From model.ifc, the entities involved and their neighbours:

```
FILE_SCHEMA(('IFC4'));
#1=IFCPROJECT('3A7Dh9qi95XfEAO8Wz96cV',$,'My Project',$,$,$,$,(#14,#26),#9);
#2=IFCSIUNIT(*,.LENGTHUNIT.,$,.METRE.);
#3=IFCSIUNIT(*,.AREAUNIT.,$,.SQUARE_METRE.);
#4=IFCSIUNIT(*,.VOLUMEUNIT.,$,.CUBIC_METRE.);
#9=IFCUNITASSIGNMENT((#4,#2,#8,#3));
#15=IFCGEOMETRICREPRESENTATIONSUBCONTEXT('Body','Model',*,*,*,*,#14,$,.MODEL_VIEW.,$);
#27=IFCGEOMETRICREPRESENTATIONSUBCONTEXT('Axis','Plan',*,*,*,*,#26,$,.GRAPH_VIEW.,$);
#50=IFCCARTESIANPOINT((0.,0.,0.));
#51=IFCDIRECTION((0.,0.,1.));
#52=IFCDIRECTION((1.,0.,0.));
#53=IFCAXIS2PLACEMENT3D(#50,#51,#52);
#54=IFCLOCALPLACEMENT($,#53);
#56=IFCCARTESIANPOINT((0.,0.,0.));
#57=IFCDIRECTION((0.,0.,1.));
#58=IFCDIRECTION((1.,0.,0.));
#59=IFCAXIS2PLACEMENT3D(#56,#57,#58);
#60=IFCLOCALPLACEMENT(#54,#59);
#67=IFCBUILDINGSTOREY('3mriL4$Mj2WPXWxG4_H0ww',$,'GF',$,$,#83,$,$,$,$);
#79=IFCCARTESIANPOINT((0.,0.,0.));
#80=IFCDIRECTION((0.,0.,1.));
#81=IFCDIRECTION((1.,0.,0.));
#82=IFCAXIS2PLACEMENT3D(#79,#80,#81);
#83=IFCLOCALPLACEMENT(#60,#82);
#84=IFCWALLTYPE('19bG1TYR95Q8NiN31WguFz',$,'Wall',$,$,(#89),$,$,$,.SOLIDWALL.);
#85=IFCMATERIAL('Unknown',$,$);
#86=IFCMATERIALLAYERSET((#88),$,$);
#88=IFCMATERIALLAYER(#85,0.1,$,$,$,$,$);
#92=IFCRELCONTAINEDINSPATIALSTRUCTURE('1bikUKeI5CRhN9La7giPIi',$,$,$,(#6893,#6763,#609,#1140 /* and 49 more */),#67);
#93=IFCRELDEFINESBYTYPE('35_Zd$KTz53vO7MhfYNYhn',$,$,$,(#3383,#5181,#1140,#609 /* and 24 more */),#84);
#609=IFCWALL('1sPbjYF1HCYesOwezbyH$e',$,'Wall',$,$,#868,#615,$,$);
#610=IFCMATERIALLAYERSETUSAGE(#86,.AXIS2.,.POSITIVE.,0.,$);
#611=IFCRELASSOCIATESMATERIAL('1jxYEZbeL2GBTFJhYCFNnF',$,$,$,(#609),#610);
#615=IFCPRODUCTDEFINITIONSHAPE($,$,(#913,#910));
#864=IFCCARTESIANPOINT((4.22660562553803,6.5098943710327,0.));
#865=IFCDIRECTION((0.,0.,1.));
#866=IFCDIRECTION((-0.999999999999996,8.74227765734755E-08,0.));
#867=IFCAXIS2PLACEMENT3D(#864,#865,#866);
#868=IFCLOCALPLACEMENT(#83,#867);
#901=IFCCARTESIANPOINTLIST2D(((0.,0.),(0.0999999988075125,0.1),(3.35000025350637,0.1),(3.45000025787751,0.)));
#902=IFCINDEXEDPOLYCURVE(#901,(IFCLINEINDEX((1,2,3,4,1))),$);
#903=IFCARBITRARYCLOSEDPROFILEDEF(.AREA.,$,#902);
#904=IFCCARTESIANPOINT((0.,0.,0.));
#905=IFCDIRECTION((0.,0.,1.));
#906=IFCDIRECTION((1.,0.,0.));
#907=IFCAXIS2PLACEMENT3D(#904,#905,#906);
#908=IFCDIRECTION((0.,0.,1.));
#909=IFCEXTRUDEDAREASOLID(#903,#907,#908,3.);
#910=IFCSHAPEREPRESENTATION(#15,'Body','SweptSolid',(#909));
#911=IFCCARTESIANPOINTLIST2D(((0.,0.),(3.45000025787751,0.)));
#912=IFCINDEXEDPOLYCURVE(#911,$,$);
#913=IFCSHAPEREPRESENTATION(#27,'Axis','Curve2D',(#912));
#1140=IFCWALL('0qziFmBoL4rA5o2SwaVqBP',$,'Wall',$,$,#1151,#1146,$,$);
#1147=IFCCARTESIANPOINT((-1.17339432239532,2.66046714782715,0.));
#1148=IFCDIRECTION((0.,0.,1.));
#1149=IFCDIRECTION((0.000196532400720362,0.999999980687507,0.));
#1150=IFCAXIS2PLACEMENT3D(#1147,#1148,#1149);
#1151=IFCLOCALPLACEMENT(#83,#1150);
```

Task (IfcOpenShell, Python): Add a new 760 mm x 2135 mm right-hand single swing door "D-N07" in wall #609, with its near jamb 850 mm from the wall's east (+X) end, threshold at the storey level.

```python
import numpy as np
import ifcopenshell
import ifcopenshell.api.feature
import ifcopenshell.api.geometry
import ifcopenshell.api.root
import ifcopenshell.api.spatial
import ifcopenshell.geom
import ifcopenshell.util.element
import ifcopenshell.util.placement
import ifcopenshell.util.representation
import ifcopenshell.util.shape
import ifcopenshell.util.unit

model = ifcopenshell.open("model.ifc")
unit_scale = ifcopenshell.util.unit.calculate_unit_scale(model)
settings = ifcopenshell.geom.settings()


def volume(element):
    """Net volume in cubic metres, openings subtracted."""
    shape = ifcopenshell.geom.create_shape(settings, element)
    return ifcopenshell.util.shape.get_volume(shape.geometry)


wall = model.by_guid("1sPbjYF1HCYesOwezbyH$e")
storey = ifcopenshell.util.element.get_container(wall, ifc_class="IfcBuildingStorey")
context = ifcopenshell.util.representation.get_context(model, "Model", "Body", "MODEL_VIEW")
before = volume(wall)

width, height, from_end, sill = 0.76, 2.135, 0.85, 0.0  # metres

# The wall runs along its own X axis, and the end named is its -X end.
wall_shape = ifcopenshell.geom.create_shape(settings, wall)
x, y, z = ifcopenshell.util.shape.get_vertices(wall_shape.geometry).T
start = x.min() + from_end
face, thickness = float(y.min()), float(y.max() - y.min())
wall_matrix = ifcopenshell.util.placement.get_local_placement(wall.ObjectPlacement)
level = ifcopenshell.util.placement.get_local_placement(storey.ObjectPlacement)[2, 3]


def in_wall(x, y):
    """Placement at x, y metres in the wall's axes, at sill height."""
    matrix = wall_matrix.copy()
    matrix[:, 3] = wall_matrix @ np.array([x / unit_scale, y / unit_scale, 0.0, 1.0])
    matrix[2, 3] = level + sill / unit_scale
    return matrix


# Opening: a box that overshoots both wall faces by 50 mm.
opening = ifcopenshell.api.root.create_entity(model, ifc_class="IfcOpeningElement", predefined_type="OPENING")
box = ifcopenshell.api.geometry.add_wall_representation(
    model, context=context, length=width, height=height, thickness=thickness + 0.1
)
ifcopenshell.api.geometry.assign_representation(model, product=opening, representation=box)
ifcopenshell.api.geometry.edit_object_placement(model, product=opening, matrix=in_wall(start, face - 0.05), is_si=False)
ifcopenshell.api.feature.add_feature(model, feature=opening, element=wall)

door = ifcopenshell.api.root.create_entity(model, ifc_class="IfcDoor", name="D-N07", predefined_type="DOOR")
door.OverallWidth, door.OverallHeight = width / unit_scale, height / unit_scale
door.OperationType = "SINGLE_SWING_RIGHT"
body = ifcopenshell.api.geometry.add_door_representation(
    model,
    context=context,
    overall_width=door.OverallWidth,
    overall_height=door.OverallHeight,
    operation_type="SINGLE_SWING_RIGHT",
    lining_properties={"LiningDepth": thickness / unit_scale, "ThresholdDepth": thickness / unit_scale},
)
ifcopenshell.api.geometry.assign_representation(model, product=door, representation=body)
ifcopenshell.api.spatial.assign_container(model, products=[door], relating_structure=storey)
ifcopenshell.api.feature.add_filling(model, opening=opening, element=door)

# The lining spans the wall, so the door starts at the wall face.
ifcopenshell.api.geometry.edit_object_placement(model, product=door, matrix=in_wall(start, face), is_si=False)

after = volume(wall)

print(f"wall volume {before:.3f} -> {after:.3f} m3")

model.write("model-out.ifc")
```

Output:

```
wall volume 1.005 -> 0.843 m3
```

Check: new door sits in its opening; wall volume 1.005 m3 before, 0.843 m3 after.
